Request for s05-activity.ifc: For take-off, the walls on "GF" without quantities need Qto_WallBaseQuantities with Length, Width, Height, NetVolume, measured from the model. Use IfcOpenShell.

First a look at what the model holds.

```python
import ifcopenshell
import ifcopenshell.util.element
import ifcopenshell.util.unit

model = ifcopenshell.open("s05-activity.ifc")
print(model.schema)
for unit_type in ("LENGTHUNIT", "AREAUNIT", "VOLUMEUNIT"):
    print(unit_type, ifcopenshell.util.unit.calculate_unit_scale(model, unit_type))
storey = next(s for s in model.by_type("IfcBuildingStorey") if s.Name == "GF")
walls = [e for e in ifcopenshell.util.element.get_decomposition(storey) if e.is_a("IfcWall")]
for e in sorted(walls, key=lambda e: e.id()):
    print(e.id(), e.is_a(), e.Name, list(ifcopenshell.util.element.get_psets(e, qtos_only=True)), sep=" | ")
```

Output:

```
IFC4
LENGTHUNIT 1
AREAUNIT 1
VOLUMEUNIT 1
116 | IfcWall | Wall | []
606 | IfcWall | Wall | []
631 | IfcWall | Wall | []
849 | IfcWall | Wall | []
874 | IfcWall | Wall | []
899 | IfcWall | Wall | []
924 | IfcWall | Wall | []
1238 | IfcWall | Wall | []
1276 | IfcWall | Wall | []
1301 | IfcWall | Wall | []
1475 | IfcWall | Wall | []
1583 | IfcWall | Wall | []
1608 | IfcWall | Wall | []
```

```python
import ifcopenshell
import ifcopenshell.api.pset
import ifcopenshell.geom
import ifcopenshell.util.element
import ifcopenshell.util.shape
import ifcopenshell.util.unit

model = ifcopenshell.open("s05-activity.ifc")
unit_scale = ifcopenshell.util.unit.calculate_unit_scale(model)
volume_scale = ifcopenshell.util.unit.calculate_unit_scale(model, "VOLUMEUNIT")
settings = ifcopenshell.geom.settings()

storey = next(s for s in model.by_type("IfcBuildingStorey") if s.Name == "GF")
walls = [e for e in ifcopenshell.util.element.get_decomposition(storey) if e.is_a("IfcWall")]

for e in sorted(walls, key=lambda e: e.id()):
    if ifcopenshell.util.element.get_psets(e, qtos_only=True, should_inherit=False):
        continue
    # Geometry comes back in metres, in the element's own axes.
    shape = ifcopenshell.geom.create_shape(settings, e)
    values = {
        "Length": ifcopenshell.util.shape.get_x(shape.geometry) / unit_scale,
        "Width": ifcopenshell.util.shape.get_y(shape.geometry) / unit_scale,
        "Height": ifcopenshell.util.shape.get_z(shape.geometry) / unit_scale,
        "NetVolume": ifcopenshell.util.shape.get_volume(shape.geometry) / volume_scale,
    }
    qto = ifcopenshell.api.pset.add_qto(model, product=e, name="Qto_WallBaseQuantities")
    ifcopenshell.api.pset.edit_qto(model, qto=qto, properties=values)
    print(e.id(), {k: round(v, 3) for k, v in values.items()})

model.write("s05-activity_v2.ifc")
```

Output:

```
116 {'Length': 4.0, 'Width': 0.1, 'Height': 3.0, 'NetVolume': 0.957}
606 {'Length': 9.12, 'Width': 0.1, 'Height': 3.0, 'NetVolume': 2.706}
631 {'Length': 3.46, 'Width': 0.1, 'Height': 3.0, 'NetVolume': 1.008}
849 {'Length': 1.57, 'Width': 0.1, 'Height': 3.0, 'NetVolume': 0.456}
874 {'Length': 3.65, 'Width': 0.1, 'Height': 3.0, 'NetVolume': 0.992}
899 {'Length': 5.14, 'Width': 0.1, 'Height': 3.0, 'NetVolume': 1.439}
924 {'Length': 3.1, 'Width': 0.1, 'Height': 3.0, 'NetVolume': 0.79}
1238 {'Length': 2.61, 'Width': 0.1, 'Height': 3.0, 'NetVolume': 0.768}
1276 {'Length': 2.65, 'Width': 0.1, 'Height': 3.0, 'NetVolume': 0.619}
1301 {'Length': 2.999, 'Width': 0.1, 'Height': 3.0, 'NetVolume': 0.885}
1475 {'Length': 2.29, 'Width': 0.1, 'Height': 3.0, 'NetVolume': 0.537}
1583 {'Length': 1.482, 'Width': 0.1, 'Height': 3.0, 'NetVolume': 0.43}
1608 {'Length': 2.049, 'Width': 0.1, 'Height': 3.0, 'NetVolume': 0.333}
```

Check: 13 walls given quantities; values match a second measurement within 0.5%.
